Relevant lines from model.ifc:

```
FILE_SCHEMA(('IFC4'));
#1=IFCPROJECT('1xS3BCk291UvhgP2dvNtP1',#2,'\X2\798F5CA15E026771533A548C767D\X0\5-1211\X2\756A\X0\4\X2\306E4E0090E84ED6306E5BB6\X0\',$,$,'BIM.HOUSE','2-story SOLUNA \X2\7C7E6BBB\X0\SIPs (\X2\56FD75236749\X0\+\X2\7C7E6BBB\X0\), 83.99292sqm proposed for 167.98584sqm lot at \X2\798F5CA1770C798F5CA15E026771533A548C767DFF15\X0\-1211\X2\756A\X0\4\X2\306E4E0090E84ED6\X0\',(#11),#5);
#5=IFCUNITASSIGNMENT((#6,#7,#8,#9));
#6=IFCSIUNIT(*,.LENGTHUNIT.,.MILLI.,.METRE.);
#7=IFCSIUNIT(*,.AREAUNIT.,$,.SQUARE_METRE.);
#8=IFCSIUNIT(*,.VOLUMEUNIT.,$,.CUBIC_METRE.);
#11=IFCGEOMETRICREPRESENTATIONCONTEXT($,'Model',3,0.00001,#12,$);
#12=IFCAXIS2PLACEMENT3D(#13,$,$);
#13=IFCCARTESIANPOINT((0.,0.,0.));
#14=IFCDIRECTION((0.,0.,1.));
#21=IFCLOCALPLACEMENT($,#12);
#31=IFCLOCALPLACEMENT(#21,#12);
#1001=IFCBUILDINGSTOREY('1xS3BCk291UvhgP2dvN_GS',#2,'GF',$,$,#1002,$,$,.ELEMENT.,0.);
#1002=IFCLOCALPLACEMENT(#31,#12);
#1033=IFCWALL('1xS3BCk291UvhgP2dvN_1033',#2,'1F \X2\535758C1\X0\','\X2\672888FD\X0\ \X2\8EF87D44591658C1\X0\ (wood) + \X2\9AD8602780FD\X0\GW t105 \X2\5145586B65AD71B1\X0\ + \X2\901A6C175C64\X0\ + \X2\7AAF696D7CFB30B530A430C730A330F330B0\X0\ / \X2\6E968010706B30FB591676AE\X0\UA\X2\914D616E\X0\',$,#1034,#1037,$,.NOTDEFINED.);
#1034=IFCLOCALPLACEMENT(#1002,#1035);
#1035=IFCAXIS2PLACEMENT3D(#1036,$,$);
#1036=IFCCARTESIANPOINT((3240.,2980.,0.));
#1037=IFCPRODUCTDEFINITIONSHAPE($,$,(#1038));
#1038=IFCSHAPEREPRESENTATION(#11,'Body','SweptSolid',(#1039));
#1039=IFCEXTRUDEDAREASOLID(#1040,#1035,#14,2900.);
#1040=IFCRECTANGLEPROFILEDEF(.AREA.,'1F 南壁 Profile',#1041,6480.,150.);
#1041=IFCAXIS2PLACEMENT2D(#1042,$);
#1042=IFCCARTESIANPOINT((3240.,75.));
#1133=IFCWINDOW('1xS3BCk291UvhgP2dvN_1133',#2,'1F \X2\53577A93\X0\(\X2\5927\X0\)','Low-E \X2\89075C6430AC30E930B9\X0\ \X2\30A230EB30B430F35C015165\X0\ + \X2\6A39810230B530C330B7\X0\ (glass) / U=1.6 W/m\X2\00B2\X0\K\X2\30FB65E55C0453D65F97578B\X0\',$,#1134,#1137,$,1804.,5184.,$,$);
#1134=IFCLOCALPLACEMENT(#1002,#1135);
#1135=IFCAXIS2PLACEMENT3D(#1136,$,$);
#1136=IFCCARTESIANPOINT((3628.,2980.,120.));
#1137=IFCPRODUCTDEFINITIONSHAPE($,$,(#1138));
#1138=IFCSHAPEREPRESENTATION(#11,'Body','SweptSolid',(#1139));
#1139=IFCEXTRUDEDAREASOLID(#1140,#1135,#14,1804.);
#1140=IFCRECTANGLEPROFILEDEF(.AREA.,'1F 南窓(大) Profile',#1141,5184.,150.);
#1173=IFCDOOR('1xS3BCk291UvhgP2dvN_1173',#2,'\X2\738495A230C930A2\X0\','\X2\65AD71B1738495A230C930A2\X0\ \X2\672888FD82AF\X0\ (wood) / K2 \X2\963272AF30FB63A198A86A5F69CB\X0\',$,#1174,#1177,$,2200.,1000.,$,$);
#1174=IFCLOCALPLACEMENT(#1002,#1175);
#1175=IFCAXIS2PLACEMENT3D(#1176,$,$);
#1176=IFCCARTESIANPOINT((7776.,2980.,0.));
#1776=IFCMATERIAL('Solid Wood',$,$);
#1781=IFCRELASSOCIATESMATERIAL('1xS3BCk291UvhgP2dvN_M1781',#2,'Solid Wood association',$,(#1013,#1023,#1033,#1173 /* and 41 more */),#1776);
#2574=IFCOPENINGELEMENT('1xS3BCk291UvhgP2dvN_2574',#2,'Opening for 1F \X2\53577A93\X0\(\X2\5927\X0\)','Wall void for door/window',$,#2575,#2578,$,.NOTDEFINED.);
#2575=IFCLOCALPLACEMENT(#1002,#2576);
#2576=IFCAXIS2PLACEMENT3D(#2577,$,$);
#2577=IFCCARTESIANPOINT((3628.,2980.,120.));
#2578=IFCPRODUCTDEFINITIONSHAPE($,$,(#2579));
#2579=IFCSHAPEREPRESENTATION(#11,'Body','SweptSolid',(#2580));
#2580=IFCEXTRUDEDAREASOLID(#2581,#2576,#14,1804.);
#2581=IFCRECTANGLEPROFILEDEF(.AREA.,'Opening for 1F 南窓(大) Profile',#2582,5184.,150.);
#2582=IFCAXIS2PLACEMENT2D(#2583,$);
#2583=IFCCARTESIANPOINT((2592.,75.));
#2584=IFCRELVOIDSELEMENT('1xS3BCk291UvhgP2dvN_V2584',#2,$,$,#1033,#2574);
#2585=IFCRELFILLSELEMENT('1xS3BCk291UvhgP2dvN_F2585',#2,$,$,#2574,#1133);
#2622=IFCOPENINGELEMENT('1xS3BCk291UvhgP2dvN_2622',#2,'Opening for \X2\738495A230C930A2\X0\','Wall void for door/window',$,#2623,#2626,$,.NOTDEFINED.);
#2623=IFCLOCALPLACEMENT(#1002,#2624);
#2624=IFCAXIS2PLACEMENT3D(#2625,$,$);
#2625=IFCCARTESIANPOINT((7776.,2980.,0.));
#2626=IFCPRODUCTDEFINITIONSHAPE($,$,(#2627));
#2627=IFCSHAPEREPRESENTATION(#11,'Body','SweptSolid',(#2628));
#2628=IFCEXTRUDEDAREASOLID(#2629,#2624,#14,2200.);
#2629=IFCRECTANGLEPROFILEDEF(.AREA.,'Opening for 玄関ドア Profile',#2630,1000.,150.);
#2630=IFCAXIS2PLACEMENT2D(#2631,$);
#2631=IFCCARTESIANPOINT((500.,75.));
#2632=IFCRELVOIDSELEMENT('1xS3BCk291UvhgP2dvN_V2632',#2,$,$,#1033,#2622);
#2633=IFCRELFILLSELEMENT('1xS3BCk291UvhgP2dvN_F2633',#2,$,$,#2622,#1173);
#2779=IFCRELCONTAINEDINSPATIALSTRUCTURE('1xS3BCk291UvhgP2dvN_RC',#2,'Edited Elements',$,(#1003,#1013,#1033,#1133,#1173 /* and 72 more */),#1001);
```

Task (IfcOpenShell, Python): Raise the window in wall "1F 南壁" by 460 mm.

```python
import numpy as np
import ifcopenshell
import ifcopenshell.api.geometry
import ifcopenshell.util.placement
import ifcopenshell.util.unit

model = ifcopenshell.open("model.ifc")
unit_scale = ifcopenshell.util.unit.calculate_unit_scale(model)

window = model.by_guid("1xS3BCk291UvhgP2dvN_1133")
opening = window.FillsVoids[0].RelatingOpeningElement
dz = 460.0

shift = np.array([0.0, 0.0, dz])
# The window is not placed relative to its opening, so move both.
for product in (opening, window):
    matrix = ifcopenshell.util.placement.get_local_placement(product.ObjectPlacement)
    matrix[:3, 3] += shift
    ifcopenshell.api.geometry.edit_object_placement(model, product=product, matrix=matrix, is_si=False)

print(f"moved by {dz * unit_scale:+.3f} m")

model.write("model_edited.ifc")
```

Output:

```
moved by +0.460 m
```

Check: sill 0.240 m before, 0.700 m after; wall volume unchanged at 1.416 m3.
